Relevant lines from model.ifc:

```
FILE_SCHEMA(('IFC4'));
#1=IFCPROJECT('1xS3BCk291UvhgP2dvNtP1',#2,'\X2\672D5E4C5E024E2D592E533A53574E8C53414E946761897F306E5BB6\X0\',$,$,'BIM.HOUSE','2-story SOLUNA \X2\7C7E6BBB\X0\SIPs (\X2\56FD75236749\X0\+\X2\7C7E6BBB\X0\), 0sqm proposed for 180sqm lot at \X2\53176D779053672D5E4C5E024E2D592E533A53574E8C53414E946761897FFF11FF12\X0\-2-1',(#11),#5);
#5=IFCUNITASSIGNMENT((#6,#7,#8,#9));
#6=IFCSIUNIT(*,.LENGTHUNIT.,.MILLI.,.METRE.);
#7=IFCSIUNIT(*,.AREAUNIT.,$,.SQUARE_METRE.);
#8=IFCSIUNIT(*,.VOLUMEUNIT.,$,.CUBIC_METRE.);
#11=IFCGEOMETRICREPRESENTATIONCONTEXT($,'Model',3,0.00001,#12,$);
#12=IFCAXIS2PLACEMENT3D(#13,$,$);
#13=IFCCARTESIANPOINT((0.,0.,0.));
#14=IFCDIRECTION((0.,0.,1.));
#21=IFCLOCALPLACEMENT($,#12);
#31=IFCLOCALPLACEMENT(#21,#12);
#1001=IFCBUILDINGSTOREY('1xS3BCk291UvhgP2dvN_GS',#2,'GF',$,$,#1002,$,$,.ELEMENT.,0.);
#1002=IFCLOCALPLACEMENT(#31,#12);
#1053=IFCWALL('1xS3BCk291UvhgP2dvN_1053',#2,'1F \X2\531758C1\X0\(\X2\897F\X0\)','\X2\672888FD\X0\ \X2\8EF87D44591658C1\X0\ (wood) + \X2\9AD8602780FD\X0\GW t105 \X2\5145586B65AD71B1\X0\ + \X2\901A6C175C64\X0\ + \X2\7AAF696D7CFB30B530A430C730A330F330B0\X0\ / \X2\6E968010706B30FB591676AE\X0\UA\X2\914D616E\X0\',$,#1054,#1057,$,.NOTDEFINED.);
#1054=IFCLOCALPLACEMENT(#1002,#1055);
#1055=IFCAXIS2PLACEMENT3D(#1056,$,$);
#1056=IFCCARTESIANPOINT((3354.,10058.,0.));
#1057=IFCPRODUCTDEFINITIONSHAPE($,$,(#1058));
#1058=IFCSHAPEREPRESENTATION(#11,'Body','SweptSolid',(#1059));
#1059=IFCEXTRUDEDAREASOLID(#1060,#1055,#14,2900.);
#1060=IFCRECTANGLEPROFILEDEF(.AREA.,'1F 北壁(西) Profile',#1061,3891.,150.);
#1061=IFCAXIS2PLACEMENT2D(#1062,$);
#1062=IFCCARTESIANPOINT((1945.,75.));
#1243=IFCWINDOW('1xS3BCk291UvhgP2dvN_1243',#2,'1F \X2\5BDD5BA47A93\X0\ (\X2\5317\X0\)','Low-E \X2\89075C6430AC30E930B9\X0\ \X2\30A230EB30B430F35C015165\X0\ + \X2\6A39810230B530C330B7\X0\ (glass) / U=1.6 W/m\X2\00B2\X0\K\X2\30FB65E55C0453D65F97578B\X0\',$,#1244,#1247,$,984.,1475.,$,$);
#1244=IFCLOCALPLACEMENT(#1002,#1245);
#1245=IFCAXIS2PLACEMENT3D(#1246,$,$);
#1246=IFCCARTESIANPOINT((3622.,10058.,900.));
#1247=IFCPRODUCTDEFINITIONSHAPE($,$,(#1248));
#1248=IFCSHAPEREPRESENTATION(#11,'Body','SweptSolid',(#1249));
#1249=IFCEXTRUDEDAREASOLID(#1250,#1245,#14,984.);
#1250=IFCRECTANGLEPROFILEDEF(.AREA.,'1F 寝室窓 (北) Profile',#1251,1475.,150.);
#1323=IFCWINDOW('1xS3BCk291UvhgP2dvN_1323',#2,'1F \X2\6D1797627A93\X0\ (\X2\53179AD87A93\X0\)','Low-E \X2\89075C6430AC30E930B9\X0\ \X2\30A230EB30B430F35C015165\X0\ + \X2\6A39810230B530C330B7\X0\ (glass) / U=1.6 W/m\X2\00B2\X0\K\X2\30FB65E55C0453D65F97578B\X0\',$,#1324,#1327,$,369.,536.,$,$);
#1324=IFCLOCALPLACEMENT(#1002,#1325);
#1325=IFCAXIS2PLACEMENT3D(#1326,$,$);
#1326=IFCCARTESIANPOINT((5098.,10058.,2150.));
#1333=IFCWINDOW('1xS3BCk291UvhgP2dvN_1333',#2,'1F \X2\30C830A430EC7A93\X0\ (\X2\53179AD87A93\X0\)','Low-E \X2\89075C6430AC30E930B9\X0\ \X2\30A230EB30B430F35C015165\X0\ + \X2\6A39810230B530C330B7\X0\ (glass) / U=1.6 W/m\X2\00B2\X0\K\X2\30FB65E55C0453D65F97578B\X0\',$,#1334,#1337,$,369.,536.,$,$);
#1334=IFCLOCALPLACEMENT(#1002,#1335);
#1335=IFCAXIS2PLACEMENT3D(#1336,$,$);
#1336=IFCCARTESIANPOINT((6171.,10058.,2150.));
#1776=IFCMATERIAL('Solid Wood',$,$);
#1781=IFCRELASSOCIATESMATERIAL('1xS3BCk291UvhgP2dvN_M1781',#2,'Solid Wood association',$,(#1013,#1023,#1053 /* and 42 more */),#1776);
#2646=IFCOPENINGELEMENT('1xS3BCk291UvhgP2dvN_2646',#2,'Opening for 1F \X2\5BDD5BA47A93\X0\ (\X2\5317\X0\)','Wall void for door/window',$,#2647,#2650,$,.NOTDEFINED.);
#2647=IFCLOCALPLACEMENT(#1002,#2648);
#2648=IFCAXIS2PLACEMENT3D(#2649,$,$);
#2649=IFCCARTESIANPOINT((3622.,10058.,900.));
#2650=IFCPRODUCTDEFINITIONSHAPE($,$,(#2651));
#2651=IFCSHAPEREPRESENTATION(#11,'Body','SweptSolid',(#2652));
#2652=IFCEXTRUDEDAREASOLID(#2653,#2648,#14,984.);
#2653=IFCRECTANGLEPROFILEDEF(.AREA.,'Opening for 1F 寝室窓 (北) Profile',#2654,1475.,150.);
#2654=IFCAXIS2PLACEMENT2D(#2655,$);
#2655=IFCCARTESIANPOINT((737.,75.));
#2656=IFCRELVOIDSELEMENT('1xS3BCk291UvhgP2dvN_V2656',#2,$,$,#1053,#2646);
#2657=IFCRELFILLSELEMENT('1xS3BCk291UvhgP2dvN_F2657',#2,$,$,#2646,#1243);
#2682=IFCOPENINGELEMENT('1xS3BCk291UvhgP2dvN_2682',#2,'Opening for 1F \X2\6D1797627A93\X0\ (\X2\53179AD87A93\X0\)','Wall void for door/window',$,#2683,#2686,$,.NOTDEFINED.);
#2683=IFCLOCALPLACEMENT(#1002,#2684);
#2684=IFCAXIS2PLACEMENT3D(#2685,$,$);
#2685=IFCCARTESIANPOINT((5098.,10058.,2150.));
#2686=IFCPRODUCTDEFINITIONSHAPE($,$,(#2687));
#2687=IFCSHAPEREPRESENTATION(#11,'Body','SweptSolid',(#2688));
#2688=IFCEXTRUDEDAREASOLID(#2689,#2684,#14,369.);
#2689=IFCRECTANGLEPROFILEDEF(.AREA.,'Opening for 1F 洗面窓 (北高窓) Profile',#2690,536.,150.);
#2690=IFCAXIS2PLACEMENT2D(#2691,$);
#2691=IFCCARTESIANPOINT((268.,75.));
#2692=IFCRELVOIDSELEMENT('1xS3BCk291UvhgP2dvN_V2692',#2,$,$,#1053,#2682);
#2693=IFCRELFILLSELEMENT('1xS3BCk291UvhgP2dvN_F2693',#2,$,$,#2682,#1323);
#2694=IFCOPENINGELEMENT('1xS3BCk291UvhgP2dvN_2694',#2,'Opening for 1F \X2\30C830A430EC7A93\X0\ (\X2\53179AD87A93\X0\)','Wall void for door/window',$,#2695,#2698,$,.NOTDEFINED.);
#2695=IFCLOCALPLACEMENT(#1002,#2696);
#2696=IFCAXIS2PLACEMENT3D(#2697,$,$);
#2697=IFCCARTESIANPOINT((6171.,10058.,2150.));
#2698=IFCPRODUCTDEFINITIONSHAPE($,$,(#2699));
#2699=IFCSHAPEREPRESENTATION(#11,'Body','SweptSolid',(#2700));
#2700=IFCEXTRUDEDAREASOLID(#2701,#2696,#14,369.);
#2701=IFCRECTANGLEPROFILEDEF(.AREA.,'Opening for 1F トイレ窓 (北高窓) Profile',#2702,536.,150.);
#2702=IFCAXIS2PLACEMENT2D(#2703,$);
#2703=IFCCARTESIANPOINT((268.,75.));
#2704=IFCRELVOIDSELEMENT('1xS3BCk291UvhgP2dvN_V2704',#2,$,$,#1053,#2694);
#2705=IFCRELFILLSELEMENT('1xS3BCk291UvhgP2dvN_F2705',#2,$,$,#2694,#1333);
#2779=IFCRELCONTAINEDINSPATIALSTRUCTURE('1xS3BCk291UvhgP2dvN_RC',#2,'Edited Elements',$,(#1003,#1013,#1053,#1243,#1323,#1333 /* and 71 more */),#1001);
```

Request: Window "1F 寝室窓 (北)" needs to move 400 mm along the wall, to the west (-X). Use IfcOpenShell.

```python
import ifcopenshell
import ifcopenshell.api.geometry
import ifcopenshell.util.placement
import ifcopenshell.util.unit

model = ifcopenshell.open("model.ifc")
unit_scale = ifcopenshell.util.unit.calculate_unit_scale(model)

window = model.by_id(1243)
opening = window.FillsVoids[0].RelatingOpeningElement
wall = opening.VoidsElements[0].RelatingBuildingElement

wall_matrix = ifcopenshell.util.placement.get_local_placement(wall.ObjectPlacement)
shift = wall_matrix[:3, 0] * -0.4 / unit_scale
before = ifcopenshell.util.placement.get_local_placement(window.ObjectPlacement)[:3, 3].copy()

# The window is not placed relative to its opening, so move both.
for product in (opening, window):
    matrix = ifcopenshell.util.placement.get_local_placement(product.ObjectPlacement)
    matrix[:3, 3] += shift
    ifcopenshell.api.geometry.edit_object_placement(model, product=product, matrix=matrix, is_si=False)

after = ifcopenshell.util.placement.get_local_placement(window.ObjectPlacement)[:3, 3]
print("window moved by", (after - before).round(3) + 0.0)

model.write("model-out.ifc")
```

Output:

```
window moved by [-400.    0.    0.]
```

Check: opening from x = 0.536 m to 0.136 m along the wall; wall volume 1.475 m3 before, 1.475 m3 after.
